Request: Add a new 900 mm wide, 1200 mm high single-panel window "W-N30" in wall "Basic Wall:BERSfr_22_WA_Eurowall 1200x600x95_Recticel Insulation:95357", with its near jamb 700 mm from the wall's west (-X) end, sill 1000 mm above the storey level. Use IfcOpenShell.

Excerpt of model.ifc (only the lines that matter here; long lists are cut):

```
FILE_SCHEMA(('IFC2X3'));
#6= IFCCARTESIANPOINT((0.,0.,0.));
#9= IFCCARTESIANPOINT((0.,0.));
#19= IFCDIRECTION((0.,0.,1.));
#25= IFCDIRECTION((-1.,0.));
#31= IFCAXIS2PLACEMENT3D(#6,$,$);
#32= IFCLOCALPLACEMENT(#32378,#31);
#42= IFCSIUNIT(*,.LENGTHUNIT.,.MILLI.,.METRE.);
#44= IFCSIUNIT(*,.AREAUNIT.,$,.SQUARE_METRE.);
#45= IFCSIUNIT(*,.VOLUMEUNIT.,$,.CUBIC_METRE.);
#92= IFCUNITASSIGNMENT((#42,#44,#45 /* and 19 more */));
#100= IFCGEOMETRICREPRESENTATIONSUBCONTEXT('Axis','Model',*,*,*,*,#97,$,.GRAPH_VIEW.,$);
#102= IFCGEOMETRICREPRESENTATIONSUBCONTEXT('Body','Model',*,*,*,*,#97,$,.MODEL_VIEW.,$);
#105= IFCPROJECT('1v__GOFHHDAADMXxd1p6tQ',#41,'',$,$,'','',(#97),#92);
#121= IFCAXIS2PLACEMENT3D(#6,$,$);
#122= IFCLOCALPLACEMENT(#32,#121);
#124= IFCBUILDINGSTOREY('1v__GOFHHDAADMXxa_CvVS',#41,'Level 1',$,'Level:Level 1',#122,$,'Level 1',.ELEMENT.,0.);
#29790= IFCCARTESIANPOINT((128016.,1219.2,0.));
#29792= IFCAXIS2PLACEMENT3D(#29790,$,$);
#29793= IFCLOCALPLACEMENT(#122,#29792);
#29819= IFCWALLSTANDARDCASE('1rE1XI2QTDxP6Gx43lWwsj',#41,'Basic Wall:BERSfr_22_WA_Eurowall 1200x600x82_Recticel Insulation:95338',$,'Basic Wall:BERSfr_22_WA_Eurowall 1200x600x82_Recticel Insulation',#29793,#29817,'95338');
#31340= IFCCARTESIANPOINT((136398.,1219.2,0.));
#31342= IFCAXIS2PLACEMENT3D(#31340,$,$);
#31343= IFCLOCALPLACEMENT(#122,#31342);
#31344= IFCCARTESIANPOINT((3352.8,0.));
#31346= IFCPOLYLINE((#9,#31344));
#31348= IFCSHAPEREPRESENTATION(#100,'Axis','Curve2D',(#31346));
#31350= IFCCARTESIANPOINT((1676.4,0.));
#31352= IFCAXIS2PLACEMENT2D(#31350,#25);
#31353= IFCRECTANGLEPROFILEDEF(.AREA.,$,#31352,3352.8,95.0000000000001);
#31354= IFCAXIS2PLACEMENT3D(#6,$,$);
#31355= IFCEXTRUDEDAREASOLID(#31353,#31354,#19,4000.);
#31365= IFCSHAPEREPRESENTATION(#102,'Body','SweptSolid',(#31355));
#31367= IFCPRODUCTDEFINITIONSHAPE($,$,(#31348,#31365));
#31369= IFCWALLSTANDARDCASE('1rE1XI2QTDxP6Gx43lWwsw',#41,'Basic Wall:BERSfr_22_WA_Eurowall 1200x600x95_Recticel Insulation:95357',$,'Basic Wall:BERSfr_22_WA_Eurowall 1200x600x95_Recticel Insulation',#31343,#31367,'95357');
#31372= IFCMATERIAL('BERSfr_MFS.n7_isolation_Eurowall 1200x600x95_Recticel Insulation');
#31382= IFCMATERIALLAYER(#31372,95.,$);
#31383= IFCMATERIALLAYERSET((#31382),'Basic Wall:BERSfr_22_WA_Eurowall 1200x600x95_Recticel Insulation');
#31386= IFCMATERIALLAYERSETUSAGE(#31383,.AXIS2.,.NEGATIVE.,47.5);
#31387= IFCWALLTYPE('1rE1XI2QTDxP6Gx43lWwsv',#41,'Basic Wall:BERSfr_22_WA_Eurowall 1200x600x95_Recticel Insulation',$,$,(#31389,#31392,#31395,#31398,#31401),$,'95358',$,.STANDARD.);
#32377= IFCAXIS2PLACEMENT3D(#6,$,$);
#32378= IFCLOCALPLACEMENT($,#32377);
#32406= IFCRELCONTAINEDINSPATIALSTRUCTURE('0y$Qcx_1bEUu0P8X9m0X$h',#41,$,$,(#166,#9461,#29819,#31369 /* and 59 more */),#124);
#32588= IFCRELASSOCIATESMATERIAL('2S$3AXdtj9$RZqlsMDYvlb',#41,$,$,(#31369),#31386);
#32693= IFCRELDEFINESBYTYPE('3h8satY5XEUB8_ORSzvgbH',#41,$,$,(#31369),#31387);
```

```python
import numpy as np
import ifcopenshell
import ifcopenshell.api.feature
import ifcopenshell.api.geometry
import ifcopenshell.api.root
import ifcopenshell.api.spatial
import ifcopenshell.api.type
import ifcopenshell.geom
import ifcopenshell.util.element
import ifcopenshell.util.placement
import ifcopenshell.util.representation
import ifcopenshell.util.shape
import ifcopenshell.util.unit

model = ifcopenshell.open("model.ifc")
unit_scale = ifcopenshell.util.unit.calculate_unit_scale(model)
settings = ifcopenshell.geom.settings()


def volume(element):
    """Net volume in cubic metres, openings subtracted."""
    shape = ifcopenshell.geom.create_shape(settings, element)
    return ifcopenshell.util.shape.get_volume(shape.geometry)


wall = model.by_id(31369)
storey = ifcopenshell.util.element.get_container(wall, ifc_class="IfcBuildingStorey")
context = ifcopenshell.util.representation.get_context(model, "Model", "Body", "MODEL_VIEW")
before = volume(wall)

width, height, from_end, sill = 0.9, 1.2, 0.7, 1  # metres

# The wall runs along its own X axis, and the end named is its -X end.
wall_shape = ifcopenshell.geom.create_shape(settings, wall)
x, y, z = ifcopenshell.util.shape.get_vertices(wall_shape.geometry).T
start = x.min() + from_end
face, thickness = float(y.min()), float(y.max() - y.min())
wall_matrix = ifcopenshell.util.placement.get_local_placement(wall.ObjectPlacement)
level = ifcopenshell.util.placement.get_local_placement(storey.ObjectPlacement)[2, 3]


def in_wall(x, y):
    """Placement at x, y metres in the wall's axes, at sill height."""
    matrix = wall_matrix.copy()
    matrix[:, 3] = wall_matrix @ np.array([x / unit_scale, y / unit_scale, 0.0, 1.0])
    matrix[2, 3] = level + sill / unit_scale
    return matrix


# Opening: a box that overshoots both wall faces by 50 mm.
opening = ifcopenshell.api.root.create_entity(model, ifc_class="IfcOpeningElement")
box = ifcopenshell.api.geometry.add_wall_representation(
    model, context=context, length=width, height=height, thickness=thickness + 0.1
)
ifcopenshell.api.geometry.assign_representation(model, product=opening, representation=box)
ifcopenshell.api.geometry.edit_object_placement(model, product=opening, matrix=in_wall(start, face - 0.05), is_si=False)
ifcopenshell.api.feature.add_feature(model, feature=opening, element=wall)

window = ifcopenshell.api.root.create_entity(model, ifc_class="IfcWindow", name="W-N30")
window.OverallWidth, window.OverallHeight = width / unit_scale, height / unit_scale
body = ifcopenshell.api.geometry.add_window_representation(
    model,
    context=context,
    overall_width=window.OverallWidth,
    overall_height=window.OverallHeight,
    partition_type="SINGLE_PANEL",
)
ifcopenshell.api.geometry.assign_representation(model, product=window, representation=body)
ifcopenshell.api.spatial.assign_container(model, products=[window], relating_structure=storey)
fills = ifcopenshell.api.feature.add_filling(model, opening=opening, element=window)
fills.OwnerHistory = window.OwnerHistory  # required in IFC2X3

# IFC2X3 keeps the operation on the window style.
style = ifcopenshell.api.root.create_entity(model, ifc_class="IfcWindowStyle", name="W-N30")
style.OperationType, style.ConstructionType = "SINGLE_PANEL", "NOTDEFINED"
style.ParameterTakesPrecedence = style.Sizeable = False
ifcopenshell.api.type.assign_type(model, related_objects=[window], relating_type=style)

# Centre the window in the wall's thickness.
ifcopenshell.api.geometry.edit_object_placement(model, product=window, matrix=in_wall(start, face), is_si=False)
window_shape = ifcopenshell.geom.create_shape(settings, window)
depth = ifcopenshell.util.shape.get_vertices(window_shape.geometry)[:, 1]
offset = face + thickness / 2 - (depth.min() + depth.max()) / 2
ifcopenshell.api.geometry.edit_object_placement(model, product=window, matrix=in_wall(start, offset), is_si=False)

after = volume(wall)

print(f"wall volume {before:.3f} -> {after:.3f} m3")

model.write("model_v2.ifc")
```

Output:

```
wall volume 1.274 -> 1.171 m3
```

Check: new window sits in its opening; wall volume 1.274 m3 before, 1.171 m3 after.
